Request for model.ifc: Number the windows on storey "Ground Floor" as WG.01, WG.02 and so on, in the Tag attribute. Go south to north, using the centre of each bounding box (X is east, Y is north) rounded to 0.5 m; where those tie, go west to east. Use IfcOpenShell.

First a look at what the model holds.

```python
import ifcopenshell
import ifcopenshell.util.element
import ifcopenshell.util.placement

model = ifcopenshell.open("model.ifc")
print(model.schema)
storey = next(s for s in model.by_type("IfcBuildingStorey") if s.Name == "Ground Floor")
windows = [e for e in ifcopenshell.util.element.get_decomposition(storey) if e.is_a("IfcWindow")]
for e in sorted(windows, key=lambda e: e.id()):
    origin = ifcopenshell.util.placement.get_local_placement(e.ObjectPlacement)[:3, 3]
    print(e.id(), e.Tag, e.Name, origin.round(2) + 0.0, sep=" | ")
```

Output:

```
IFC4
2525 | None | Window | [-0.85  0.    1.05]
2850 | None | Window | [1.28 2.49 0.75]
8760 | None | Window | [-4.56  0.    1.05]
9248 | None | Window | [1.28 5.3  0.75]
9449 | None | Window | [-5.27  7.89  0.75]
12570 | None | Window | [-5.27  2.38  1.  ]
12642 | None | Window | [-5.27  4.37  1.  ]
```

```python
import ifcopenshell
import ifcopenshell.geom
import ifcopenshell.util.element
import ifcopenshell.util.shape

model = ifcopenshell.open("model.ifc")
settings = ifcopenshell.geom.settings()
settings.set("use-world-coords", True)


def centre(element):
    shape = ifcopenshell.geom.create_shape(settings, element)
    return ifcopenshell.util.shape.get_bbox_centroid(shape.geometry)


storey = next(s for s in model.by_type("IfcBuildingStorey") if s.Name == "Ground Floor")
windows = [e for e in ifcopenshell.util.element.get_decomposition(storey) if e.is_a("IfcWindow")]

# Insertion points can sit at a corner or the storey origin, so sort by the geometry (in metres).
centres = {e: centre(e) for e in windows}
windows.sort(key=lambda e: (round(centres[e][1] / 0.5), centres[e][0]))

for i, e in enumerate(windows, start=1):
    number = f"WG.{i:02d}"
    e.Tag = number
    print(e.id(), number)

model.write("model_rev.ifc")
```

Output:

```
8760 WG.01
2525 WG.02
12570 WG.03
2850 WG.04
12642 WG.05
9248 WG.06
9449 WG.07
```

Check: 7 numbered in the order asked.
